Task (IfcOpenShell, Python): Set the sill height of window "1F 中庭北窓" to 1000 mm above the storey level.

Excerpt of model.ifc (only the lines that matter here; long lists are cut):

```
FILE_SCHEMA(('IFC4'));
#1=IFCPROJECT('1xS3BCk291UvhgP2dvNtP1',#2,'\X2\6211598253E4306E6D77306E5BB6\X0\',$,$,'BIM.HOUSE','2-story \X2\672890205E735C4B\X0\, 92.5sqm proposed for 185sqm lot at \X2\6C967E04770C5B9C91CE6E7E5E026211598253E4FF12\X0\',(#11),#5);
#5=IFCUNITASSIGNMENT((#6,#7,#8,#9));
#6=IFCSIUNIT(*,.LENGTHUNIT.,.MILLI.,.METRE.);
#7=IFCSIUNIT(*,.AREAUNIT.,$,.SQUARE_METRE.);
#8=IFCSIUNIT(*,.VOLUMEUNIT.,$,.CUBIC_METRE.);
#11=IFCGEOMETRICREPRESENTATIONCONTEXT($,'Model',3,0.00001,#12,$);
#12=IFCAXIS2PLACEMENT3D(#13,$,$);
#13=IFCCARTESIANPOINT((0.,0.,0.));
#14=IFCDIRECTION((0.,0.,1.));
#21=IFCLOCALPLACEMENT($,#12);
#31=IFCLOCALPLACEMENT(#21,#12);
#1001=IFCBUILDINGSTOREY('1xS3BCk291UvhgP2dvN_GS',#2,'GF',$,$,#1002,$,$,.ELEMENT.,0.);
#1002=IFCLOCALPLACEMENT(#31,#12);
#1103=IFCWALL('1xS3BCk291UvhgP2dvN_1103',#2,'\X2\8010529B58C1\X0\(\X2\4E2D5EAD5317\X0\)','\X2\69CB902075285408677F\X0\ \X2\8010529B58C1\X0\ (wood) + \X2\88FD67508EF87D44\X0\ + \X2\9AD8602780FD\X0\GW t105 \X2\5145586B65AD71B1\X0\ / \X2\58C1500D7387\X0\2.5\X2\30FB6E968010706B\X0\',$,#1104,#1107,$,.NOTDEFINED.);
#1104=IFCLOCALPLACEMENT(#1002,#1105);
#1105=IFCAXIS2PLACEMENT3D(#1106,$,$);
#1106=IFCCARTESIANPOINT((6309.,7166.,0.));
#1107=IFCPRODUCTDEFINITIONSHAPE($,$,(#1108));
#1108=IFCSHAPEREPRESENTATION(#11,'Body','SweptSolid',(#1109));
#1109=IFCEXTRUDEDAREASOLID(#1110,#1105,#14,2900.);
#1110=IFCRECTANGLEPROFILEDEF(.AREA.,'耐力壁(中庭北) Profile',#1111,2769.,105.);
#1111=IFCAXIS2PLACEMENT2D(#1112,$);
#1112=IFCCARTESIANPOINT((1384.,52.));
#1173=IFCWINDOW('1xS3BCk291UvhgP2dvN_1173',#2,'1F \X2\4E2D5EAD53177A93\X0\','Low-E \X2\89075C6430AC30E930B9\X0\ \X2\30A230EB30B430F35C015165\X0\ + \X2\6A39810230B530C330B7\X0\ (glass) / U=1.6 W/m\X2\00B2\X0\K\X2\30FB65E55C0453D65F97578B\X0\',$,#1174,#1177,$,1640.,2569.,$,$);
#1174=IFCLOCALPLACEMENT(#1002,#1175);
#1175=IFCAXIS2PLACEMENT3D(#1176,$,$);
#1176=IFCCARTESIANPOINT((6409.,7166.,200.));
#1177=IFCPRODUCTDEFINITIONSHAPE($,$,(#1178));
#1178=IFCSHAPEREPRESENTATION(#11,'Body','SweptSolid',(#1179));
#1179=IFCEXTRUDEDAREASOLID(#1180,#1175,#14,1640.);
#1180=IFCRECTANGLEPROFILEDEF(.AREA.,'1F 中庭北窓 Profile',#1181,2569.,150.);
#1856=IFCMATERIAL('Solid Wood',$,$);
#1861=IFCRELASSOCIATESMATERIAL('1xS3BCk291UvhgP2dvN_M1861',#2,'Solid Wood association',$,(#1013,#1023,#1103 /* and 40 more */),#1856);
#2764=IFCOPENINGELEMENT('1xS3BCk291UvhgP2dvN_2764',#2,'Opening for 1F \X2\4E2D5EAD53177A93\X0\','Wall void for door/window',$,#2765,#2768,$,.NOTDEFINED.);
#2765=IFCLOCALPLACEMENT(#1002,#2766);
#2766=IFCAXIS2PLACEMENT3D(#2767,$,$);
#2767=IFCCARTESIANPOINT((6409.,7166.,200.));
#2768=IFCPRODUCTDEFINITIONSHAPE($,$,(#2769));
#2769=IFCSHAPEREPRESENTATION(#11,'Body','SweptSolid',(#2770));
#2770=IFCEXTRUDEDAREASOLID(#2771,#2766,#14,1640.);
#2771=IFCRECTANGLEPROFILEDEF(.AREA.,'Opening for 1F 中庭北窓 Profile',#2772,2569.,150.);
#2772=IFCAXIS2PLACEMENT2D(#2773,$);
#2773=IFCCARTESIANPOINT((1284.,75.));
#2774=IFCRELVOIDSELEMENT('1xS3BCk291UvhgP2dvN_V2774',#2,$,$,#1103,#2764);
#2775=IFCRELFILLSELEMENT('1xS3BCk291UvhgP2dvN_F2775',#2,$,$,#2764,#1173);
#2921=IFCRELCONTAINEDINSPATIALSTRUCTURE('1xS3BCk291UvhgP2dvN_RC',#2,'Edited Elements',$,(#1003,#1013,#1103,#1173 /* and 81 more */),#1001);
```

```python
import numpy as np
import ifcopenshell
import ifcopenshell.api.geometry
import ifcopenshell.geom
import ifcopenshell.util.element
import ifcopenshell.util.placement
import ifcopenshell.util.shape
import ifcopenshell.util.unit

model = ifcopenshell.open("model.ifc")
unit_scale = ifcopenshell.util.unit.calculate_unit_scale(model)

window = model.by_guid("1xS3BCk291UvhgP2dvN_1173")
opening = window.FillsVoids[0].RelatingOpeningElement
storey = ifcopenshell.util.element.get_container(window, ifc_class="IfcBuildingStorey")
level = ifcopenshell.util.placement.get_local_placement(storey.ObjectPlacement)[2, 3]

# The opening's origin need not be at the sill, so measure its lowest point.
shape = ifcopenshell.geom.create_shape(ifcopenshell.geom.settings(), opening)
bottom = ifcopenshell.util.shape.get_shape_bottom_elevation(shape, shape.geometry) / unit_scale
dz = level + 1000.0 - bottom

shift = np.array([0.0, 0.0, dz])
# The window is not placed relative to its opening, so move both.
for product in (opening, window):
    matrix = ifcopenshell.util.placement.get_local_placement(product.ObjectPlacement)
    matrix[:3, 3] += shift
    ifcopenshell.api.geometry.edit_object_placement(model, product=product, matrix=matrix, is_si=False)

print(f"moved by {dz * unit_scale:+.3f} m")

model.write("model_v2.ifc")
```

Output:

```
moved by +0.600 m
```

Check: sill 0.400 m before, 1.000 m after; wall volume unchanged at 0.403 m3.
